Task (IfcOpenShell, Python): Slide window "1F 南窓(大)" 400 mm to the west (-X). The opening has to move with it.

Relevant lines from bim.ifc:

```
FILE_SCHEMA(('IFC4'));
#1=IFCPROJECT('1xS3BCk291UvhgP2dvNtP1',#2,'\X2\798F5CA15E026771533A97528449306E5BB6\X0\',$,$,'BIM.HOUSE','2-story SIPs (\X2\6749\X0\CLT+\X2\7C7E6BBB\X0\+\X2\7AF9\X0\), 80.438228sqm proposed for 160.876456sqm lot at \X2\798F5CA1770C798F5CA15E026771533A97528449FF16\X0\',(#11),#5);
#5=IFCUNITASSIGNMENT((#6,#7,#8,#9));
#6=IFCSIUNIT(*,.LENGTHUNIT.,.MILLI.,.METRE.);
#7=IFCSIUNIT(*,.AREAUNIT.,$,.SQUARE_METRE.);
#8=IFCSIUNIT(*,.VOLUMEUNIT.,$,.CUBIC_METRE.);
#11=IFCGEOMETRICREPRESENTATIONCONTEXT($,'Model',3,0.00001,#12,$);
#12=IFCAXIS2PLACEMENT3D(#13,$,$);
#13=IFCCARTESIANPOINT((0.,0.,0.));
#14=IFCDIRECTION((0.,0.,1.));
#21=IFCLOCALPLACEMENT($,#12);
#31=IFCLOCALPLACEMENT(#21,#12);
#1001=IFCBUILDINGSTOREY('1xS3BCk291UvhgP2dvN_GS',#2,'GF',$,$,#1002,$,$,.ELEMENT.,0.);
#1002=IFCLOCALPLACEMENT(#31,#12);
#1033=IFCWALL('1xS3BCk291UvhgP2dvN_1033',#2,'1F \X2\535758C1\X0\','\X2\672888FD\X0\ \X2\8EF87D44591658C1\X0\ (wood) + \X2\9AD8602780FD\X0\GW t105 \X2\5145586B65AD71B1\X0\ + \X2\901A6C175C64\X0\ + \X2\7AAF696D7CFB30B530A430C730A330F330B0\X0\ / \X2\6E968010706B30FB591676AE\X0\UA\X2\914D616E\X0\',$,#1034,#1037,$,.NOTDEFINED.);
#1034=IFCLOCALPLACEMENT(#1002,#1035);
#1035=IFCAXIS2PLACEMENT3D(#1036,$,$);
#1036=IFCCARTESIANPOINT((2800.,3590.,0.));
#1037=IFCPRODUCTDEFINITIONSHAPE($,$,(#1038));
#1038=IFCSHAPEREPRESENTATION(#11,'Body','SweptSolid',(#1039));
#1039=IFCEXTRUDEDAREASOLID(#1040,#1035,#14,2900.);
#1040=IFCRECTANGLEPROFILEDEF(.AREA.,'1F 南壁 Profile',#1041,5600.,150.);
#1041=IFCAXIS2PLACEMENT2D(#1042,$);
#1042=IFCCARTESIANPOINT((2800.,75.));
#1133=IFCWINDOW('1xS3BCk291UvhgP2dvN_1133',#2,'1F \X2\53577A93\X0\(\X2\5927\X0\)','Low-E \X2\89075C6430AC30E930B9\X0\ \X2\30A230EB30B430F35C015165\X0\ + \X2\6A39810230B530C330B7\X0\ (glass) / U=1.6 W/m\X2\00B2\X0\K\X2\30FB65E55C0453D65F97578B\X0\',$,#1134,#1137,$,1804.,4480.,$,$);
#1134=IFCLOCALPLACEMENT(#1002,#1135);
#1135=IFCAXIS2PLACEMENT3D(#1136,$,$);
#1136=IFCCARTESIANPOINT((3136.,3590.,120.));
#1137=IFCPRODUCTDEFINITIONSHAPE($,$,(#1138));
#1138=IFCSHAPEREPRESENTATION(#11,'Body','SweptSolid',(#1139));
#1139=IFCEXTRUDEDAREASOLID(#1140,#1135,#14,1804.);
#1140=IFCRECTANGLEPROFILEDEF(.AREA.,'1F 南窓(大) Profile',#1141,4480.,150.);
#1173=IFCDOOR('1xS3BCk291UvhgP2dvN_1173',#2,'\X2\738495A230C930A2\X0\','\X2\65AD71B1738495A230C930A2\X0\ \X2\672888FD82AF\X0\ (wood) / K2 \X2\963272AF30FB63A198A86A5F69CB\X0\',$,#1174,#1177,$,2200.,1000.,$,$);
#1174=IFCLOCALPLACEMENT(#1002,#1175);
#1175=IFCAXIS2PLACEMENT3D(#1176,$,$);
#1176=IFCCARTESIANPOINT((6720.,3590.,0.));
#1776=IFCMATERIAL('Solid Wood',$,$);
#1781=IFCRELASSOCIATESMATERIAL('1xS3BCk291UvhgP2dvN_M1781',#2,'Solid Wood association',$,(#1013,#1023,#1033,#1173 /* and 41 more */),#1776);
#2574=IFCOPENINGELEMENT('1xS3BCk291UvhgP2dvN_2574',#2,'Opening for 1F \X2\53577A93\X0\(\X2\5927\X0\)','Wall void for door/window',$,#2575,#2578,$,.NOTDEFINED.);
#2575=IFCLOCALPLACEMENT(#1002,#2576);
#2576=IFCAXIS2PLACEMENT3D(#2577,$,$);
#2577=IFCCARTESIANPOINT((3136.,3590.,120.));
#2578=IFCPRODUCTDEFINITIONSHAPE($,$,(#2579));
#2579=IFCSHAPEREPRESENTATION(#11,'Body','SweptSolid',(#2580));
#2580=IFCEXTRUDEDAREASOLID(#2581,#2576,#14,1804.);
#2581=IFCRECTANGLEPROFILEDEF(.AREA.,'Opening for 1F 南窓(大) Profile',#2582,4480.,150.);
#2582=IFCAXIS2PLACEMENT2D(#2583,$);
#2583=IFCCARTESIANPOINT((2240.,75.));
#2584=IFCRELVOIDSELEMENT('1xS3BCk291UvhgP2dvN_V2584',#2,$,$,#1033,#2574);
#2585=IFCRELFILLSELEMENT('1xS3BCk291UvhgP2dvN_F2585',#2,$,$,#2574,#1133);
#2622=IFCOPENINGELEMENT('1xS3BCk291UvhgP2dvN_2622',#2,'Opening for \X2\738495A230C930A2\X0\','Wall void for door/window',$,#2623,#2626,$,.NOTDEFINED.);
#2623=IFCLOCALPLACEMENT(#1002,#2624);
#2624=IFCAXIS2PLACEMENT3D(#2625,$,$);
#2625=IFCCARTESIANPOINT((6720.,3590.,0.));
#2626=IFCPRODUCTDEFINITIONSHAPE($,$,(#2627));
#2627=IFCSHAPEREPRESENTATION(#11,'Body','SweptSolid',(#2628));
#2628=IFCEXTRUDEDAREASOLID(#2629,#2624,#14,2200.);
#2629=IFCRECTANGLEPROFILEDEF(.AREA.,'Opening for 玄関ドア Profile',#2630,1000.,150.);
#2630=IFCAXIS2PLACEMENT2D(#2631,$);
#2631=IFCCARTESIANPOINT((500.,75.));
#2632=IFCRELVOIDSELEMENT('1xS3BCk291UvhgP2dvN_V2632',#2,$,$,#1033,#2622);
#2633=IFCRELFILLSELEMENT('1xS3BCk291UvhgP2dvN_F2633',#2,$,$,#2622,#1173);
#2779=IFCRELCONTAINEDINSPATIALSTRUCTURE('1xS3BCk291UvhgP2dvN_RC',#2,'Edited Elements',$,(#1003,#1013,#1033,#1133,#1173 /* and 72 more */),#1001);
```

```python
import ifcopenshell
import ifcopenshell.api.geometry
import ifcopenshell.util.placement

model = ifcopenshell.open("bim.ifc")

window = model.by_id(1133)
opening = window.FillsVoids[0].RelatingOpeningElement
wall = opening.VoidsElements[0].RelatingBuildingElement

wall_matrix = ifcopenshell.util.placement.get_local_placement(wall.ObjectPlacement)
shift = wall_matrix[:3, 0] * -400.0
before = ifcopenshell.util.placement.get_local_placement(window.ObjectPlacement)[:3, 3].copy()

# The window is not placed relative to its opening, so move both.
for product in (opening, window):
    matrix = ifcopenshell.util.placement.get_local_placement(product.ObjectPlacement)
    matrix[:3, 3] += shift
    ifcopenshell.api.geometry.edit_object_placement(model, product=product, matrix=matrix, is_si=False)

after = ifcopenshell.util.placement.get_local_placement(window.ObjectPlacement)[:3, 3]
print("window moved by", (after - before).round(3) + 0.0)

model.write("bim_rev.ifc")
```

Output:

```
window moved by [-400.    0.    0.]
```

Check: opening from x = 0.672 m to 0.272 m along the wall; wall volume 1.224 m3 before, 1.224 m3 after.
